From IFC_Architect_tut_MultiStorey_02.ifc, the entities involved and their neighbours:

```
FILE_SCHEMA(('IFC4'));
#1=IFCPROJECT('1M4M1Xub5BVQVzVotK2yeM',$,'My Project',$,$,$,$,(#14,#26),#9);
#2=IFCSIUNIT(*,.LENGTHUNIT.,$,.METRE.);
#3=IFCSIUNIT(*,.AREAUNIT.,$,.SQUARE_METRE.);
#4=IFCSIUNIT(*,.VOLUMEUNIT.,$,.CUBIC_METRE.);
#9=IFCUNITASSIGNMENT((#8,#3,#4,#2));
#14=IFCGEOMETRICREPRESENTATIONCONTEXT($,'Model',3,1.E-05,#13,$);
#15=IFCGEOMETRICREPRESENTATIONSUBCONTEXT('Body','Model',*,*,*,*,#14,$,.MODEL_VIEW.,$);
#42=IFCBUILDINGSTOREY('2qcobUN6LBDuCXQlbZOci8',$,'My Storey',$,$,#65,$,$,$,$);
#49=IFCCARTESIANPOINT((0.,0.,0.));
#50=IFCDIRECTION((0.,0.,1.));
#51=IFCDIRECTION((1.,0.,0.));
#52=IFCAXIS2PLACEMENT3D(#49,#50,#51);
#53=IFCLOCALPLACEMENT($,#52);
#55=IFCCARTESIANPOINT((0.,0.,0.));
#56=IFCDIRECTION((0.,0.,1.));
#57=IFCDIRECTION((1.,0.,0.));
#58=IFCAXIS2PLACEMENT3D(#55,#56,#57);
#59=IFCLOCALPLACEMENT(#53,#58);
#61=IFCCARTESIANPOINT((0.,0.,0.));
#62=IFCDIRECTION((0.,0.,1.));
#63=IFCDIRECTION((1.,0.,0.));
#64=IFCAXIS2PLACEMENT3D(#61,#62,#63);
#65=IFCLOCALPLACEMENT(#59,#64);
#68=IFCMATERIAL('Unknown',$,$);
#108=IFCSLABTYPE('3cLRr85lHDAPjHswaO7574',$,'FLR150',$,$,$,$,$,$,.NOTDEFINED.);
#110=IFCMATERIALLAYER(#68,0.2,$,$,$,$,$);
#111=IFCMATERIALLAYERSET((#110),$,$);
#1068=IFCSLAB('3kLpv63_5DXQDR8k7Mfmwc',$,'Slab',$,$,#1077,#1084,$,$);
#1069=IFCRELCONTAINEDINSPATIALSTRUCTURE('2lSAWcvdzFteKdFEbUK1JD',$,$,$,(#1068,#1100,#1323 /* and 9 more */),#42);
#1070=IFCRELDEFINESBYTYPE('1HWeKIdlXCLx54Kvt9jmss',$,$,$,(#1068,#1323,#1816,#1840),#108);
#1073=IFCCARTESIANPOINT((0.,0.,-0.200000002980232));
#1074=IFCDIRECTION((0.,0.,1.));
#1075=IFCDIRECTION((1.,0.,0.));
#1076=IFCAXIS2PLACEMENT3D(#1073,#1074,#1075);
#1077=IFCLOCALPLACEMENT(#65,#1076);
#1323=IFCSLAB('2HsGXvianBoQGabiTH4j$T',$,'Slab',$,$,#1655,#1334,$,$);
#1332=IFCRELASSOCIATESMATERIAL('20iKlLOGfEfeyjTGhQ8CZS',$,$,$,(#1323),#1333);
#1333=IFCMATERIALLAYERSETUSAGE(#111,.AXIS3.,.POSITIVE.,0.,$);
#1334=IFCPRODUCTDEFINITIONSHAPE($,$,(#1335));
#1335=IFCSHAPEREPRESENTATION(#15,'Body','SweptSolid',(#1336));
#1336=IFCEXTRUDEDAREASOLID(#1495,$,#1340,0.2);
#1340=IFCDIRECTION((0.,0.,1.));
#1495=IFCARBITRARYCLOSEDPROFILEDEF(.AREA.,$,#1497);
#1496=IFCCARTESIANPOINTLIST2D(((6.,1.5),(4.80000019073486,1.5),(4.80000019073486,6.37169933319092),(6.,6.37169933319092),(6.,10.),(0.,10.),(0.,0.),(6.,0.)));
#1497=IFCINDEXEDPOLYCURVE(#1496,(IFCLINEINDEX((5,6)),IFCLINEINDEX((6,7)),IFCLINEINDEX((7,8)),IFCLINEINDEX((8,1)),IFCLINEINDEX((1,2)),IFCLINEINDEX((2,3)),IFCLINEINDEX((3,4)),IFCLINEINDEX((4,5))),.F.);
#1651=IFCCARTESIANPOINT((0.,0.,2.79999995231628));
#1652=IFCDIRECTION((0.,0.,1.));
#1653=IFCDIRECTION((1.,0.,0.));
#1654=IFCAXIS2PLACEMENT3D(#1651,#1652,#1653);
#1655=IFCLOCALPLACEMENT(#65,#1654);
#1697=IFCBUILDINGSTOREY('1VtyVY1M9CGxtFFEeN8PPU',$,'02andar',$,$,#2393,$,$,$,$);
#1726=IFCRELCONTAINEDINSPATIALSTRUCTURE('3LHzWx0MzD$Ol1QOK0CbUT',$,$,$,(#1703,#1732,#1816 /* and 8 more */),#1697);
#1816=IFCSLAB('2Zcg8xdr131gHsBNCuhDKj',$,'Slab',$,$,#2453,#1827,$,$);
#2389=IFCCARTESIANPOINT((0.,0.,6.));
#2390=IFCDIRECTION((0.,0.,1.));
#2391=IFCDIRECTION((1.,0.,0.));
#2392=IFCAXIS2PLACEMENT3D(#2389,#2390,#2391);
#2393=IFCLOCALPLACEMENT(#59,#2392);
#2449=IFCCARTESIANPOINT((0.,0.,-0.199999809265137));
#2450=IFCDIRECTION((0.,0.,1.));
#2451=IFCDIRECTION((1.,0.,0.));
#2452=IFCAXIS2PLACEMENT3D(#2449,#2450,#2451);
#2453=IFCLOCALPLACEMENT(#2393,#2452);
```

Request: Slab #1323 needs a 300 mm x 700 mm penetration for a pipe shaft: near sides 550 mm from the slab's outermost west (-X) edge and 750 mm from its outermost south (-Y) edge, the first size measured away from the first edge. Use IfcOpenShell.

```python
import numpy as np
import ifcopenshell
import ifcopenshell.api.feature
import ifcopenshell.api.geometry
import ifcopenshell.api.root
import ifcopenshell.geom
import ifcopenshell.util.placement
import ifcopenshell.util.representation
import ifcopenshell.util.shape
import ifcopenshell.util.unit

model = ifcopenshell.open("IFC_Architect_tut_MultiStorey_02.ifc")
unit_scale = ifcopenshell.util.unit.calculate_unit_scale(model)
settings = ifcopenshell.geom.settings()


def volume(element):
    """Net volume in cubic metres, openings subtracted."""
    shape = ifcopenshell.geom.create_shape(settings, element)
    return ifcopenshell.util.shape.get_volume(shape.geometry)


slab = model.by_id(1323)
before = volume(slab)

# Extent in the slab's own axes, in metres. The edges named are its -X and -Y sides.
slab_shape = ifcopenshell.geom.create_shape(settings, slab)
vertices = ifcopenshell.util.shape.get_vertices(slab_shape.geometry)
x_min, y_min, bottom = vertices.min(axis=0)
top = vertices[:, 2].max()

opening = ifcopenshell.api.root.create_entity(model, ifc_class="IfcOpeningElement", name="Pipe shaft opening", predefined_type="OPENING")
context = ifcopenshell.util.representation.get_context(model, "Model", "Body", "MODEL_VIEW")
width, depth = 0.3, 0.7
outline = [(0.0, 0.0), (width, 0.0), (width, depth), (0.0, depth), (0.0, 0.0)]
# Overshoot both faces by 50 mm so the cut is clean.
shape = ifcopenshell.api.geometry.add_slab_representation(
    model, context=context, depth=top - bottom + 0.1, polyline=outline
)
ifcopenshell.api.geometry.assign_representation(model, product=opening, representation=shape)

matrix = ifcopenshell.util.placement.get_local_placement(slab.ObjectPlacement)
matrix[:, 3] = matrix @ np.append(np.array([x_min + 0.55, y_min + 0.75, bottom - 0.05]) / unit_scale, 1.0)
ifcopenshell.api.geometry.edit_object_placement(model, product=opening, matrix=matrix, is_si=False)
ifcopenshell.api.feature.add_feature(model, feature=opening, element=slab)

after = volume(slab)

print(f"slab volume {before:.3f} -> {after:.3f} m3")

model.write("IFC_Architect_tut_MultiStorey_02_updated.ifc")
```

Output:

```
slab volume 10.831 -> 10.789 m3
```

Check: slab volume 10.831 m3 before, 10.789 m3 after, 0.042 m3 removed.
